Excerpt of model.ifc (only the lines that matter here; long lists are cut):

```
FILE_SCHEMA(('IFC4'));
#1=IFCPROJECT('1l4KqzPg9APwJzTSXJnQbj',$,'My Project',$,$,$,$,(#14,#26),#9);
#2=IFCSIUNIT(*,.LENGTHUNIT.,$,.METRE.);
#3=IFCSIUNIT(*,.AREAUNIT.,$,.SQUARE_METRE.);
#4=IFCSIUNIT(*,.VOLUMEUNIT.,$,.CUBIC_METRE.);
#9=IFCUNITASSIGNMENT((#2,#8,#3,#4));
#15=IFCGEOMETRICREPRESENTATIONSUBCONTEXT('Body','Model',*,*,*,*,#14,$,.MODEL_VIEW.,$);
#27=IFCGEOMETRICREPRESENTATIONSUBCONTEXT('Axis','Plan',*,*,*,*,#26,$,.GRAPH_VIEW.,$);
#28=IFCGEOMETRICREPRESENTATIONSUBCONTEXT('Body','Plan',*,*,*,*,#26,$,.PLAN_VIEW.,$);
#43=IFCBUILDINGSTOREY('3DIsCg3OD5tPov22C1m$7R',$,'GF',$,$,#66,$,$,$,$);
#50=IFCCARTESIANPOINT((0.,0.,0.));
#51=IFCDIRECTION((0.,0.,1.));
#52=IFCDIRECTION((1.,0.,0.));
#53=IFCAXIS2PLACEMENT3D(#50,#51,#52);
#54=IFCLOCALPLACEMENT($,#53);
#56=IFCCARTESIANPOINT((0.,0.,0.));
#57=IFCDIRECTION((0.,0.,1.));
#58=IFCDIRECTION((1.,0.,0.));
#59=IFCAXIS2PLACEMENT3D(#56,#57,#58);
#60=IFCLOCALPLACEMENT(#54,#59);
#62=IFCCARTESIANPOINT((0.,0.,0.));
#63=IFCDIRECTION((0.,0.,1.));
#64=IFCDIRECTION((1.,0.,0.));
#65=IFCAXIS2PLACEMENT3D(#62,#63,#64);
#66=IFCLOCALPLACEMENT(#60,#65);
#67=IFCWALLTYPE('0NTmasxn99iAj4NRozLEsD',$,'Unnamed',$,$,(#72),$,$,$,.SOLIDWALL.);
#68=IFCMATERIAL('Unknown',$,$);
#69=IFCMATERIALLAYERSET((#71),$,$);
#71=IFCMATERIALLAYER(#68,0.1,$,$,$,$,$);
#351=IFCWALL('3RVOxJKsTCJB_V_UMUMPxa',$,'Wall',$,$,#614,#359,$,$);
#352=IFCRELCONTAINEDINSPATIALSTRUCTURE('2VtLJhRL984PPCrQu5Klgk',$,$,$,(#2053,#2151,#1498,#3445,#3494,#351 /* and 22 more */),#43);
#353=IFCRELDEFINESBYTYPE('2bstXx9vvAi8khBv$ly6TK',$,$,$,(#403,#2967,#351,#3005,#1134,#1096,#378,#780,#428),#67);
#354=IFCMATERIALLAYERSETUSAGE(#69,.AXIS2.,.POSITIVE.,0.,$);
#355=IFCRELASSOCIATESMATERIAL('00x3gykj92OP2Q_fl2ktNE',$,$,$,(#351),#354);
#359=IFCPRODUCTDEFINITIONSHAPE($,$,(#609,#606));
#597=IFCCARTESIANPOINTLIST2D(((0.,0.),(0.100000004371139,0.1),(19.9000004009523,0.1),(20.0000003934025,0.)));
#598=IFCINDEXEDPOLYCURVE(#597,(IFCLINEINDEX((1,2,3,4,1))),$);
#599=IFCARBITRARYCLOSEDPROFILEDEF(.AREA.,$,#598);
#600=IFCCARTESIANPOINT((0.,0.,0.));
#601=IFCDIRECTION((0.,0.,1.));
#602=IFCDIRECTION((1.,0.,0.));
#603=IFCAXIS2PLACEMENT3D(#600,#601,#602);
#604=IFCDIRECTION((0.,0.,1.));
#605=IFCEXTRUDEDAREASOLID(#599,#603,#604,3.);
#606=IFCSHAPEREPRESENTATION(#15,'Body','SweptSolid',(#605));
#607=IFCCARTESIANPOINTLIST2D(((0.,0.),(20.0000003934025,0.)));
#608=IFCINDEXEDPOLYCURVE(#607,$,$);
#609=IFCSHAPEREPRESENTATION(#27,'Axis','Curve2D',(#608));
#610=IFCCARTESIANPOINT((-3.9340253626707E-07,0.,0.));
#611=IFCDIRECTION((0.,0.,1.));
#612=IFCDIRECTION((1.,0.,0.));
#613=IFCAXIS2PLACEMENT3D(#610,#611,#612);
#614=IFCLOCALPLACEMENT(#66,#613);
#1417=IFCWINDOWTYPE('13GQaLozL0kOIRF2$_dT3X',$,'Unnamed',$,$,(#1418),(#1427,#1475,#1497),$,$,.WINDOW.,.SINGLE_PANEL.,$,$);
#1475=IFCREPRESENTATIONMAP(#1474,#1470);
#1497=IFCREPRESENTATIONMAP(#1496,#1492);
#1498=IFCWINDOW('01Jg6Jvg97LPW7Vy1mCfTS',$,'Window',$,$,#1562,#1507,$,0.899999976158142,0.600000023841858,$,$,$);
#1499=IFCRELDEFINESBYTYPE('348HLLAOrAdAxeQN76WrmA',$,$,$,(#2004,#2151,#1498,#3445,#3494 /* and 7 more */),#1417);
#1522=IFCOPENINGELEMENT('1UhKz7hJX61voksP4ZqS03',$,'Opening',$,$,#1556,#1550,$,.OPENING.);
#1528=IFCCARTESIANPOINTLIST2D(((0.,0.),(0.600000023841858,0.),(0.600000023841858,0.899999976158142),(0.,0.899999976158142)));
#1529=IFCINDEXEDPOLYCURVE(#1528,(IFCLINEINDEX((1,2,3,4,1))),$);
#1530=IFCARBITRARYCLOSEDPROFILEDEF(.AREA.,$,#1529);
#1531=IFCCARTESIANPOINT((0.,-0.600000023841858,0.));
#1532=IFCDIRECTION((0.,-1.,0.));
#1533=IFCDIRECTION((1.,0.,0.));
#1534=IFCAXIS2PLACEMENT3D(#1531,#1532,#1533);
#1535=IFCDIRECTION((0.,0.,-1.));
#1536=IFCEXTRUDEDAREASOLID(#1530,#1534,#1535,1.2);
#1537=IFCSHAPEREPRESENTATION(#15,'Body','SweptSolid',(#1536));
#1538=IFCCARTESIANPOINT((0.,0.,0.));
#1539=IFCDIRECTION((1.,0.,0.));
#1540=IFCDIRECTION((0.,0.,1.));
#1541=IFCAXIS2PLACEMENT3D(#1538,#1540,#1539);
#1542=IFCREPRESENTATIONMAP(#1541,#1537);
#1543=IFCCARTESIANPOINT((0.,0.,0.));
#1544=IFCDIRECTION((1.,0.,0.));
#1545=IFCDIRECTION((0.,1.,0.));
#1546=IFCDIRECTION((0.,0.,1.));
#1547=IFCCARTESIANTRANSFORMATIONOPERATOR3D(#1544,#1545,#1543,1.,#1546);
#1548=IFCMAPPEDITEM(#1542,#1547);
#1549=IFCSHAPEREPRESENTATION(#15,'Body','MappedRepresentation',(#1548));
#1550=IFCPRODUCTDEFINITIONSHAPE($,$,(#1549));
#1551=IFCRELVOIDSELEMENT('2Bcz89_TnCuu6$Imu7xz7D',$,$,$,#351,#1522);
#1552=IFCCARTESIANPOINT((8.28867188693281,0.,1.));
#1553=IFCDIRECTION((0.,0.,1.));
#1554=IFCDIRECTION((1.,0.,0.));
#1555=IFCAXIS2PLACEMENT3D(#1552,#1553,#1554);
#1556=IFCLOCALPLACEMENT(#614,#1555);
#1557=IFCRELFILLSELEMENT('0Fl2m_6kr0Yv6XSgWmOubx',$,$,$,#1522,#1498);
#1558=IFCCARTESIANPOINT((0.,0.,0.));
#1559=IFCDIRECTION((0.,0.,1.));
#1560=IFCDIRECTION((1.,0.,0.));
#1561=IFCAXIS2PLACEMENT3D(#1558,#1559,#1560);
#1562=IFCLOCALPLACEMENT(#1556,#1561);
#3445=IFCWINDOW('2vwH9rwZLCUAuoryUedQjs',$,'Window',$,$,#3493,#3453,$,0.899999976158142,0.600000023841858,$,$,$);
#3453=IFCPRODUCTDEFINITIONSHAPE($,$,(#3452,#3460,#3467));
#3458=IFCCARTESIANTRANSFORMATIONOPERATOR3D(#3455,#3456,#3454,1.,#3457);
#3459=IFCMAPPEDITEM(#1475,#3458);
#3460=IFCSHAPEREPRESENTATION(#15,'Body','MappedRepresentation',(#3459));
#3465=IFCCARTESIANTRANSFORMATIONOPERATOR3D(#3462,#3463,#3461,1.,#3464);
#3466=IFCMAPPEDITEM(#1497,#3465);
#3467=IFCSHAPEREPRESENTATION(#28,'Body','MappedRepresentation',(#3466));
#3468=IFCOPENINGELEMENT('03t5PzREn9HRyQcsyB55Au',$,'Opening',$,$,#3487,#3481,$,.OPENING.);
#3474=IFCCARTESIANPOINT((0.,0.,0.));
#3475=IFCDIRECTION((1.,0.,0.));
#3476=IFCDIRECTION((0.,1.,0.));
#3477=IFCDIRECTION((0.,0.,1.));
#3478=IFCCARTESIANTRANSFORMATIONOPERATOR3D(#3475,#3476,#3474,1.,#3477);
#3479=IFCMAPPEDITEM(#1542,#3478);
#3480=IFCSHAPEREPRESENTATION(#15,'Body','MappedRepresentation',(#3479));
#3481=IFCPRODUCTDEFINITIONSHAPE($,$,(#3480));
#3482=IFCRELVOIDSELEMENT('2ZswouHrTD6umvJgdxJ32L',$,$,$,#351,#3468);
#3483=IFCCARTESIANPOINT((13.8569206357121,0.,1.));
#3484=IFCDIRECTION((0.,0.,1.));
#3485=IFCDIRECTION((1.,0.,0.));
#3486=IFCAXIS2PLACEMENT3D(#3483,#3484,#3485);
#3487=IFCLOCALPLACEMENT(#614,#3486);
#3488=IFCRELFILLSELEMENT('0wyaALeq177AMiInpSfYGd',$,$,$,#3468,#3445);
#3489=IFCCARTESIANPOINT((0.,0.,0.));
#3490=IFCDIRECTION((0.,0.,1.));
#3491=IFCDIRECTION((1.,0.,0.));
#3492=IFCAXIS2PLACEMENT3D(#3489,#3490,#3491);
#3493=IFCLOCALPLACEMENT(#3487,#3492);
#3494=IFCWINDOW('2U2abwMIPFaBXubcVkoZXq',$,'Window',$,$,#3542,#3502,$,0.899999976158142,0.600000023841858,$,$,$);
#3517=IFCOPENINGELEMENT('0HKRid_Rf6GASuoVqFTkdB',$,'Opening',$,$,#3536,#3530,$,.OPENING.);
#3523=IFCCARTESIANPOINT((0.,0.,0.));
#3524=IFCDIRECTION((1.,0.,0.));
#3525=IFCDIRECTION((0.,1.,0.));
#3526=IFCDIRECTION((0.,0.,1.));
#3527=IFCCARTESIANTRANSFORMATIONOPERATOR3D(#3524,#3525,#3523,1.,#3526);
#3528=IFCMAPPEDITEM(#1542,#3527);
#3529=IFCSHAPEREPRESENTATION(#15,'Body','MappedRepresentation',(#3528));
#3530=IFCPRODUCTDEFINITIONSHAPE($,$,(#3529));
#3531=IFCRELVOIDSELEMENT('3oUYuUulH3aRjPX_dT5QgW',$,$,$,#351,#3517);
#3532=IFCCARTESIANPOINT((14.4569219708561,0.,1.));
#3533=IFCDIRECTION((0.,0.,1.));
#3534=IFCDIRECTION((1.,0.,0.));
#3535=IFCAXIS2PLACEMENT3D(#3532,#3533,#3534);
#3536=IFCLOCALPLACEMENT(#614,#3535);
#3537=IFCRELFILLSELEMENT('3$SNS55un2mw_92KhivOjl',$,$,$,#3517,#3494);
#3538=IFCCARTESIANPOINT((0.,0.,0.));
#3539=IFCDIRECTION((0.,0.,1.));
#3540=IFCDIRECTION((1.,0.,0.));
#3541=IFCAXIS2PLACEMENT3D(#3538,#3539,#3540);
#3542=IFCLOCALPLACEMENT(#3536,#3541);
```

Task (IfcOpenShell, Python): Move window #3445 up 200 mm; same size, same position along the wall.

```python
import numpy as np
import ifcopenshell
import ifcopenshell.api.geometry
import ifcopenshell.util.placement
import ifcopenshell.util.unit

model = ifcopenshell.open("model.ifc")
unit_scale = ifcopenshell.util.unit.calculate_unit_scale(model)

window = model.by_id(3445)
opening = window.FillsVoids[0].RelatingOpeningElement
dz = 0.2 / unit_scale

shift = np.array([0.0, 0.0, dz])
# The window is placed relative to its opening, so it follows when the opening moves.
matrix = ifcopenshell.util.placement.get_local_placement(opening.ObjectPlacement)
matrix[:3, 3] += shift
ifcopenshell.api.geometry.edit_object_placement(
    model, product=opening, matrix=matrix, is_si=False, should_transform_children=True
)

print(f"moved by {dz * unit_scale:+.3f} m")

model.write("model_edited.ifc")
```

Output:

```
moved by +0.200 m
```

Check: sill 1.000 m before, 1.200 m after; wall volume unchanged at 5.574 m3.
